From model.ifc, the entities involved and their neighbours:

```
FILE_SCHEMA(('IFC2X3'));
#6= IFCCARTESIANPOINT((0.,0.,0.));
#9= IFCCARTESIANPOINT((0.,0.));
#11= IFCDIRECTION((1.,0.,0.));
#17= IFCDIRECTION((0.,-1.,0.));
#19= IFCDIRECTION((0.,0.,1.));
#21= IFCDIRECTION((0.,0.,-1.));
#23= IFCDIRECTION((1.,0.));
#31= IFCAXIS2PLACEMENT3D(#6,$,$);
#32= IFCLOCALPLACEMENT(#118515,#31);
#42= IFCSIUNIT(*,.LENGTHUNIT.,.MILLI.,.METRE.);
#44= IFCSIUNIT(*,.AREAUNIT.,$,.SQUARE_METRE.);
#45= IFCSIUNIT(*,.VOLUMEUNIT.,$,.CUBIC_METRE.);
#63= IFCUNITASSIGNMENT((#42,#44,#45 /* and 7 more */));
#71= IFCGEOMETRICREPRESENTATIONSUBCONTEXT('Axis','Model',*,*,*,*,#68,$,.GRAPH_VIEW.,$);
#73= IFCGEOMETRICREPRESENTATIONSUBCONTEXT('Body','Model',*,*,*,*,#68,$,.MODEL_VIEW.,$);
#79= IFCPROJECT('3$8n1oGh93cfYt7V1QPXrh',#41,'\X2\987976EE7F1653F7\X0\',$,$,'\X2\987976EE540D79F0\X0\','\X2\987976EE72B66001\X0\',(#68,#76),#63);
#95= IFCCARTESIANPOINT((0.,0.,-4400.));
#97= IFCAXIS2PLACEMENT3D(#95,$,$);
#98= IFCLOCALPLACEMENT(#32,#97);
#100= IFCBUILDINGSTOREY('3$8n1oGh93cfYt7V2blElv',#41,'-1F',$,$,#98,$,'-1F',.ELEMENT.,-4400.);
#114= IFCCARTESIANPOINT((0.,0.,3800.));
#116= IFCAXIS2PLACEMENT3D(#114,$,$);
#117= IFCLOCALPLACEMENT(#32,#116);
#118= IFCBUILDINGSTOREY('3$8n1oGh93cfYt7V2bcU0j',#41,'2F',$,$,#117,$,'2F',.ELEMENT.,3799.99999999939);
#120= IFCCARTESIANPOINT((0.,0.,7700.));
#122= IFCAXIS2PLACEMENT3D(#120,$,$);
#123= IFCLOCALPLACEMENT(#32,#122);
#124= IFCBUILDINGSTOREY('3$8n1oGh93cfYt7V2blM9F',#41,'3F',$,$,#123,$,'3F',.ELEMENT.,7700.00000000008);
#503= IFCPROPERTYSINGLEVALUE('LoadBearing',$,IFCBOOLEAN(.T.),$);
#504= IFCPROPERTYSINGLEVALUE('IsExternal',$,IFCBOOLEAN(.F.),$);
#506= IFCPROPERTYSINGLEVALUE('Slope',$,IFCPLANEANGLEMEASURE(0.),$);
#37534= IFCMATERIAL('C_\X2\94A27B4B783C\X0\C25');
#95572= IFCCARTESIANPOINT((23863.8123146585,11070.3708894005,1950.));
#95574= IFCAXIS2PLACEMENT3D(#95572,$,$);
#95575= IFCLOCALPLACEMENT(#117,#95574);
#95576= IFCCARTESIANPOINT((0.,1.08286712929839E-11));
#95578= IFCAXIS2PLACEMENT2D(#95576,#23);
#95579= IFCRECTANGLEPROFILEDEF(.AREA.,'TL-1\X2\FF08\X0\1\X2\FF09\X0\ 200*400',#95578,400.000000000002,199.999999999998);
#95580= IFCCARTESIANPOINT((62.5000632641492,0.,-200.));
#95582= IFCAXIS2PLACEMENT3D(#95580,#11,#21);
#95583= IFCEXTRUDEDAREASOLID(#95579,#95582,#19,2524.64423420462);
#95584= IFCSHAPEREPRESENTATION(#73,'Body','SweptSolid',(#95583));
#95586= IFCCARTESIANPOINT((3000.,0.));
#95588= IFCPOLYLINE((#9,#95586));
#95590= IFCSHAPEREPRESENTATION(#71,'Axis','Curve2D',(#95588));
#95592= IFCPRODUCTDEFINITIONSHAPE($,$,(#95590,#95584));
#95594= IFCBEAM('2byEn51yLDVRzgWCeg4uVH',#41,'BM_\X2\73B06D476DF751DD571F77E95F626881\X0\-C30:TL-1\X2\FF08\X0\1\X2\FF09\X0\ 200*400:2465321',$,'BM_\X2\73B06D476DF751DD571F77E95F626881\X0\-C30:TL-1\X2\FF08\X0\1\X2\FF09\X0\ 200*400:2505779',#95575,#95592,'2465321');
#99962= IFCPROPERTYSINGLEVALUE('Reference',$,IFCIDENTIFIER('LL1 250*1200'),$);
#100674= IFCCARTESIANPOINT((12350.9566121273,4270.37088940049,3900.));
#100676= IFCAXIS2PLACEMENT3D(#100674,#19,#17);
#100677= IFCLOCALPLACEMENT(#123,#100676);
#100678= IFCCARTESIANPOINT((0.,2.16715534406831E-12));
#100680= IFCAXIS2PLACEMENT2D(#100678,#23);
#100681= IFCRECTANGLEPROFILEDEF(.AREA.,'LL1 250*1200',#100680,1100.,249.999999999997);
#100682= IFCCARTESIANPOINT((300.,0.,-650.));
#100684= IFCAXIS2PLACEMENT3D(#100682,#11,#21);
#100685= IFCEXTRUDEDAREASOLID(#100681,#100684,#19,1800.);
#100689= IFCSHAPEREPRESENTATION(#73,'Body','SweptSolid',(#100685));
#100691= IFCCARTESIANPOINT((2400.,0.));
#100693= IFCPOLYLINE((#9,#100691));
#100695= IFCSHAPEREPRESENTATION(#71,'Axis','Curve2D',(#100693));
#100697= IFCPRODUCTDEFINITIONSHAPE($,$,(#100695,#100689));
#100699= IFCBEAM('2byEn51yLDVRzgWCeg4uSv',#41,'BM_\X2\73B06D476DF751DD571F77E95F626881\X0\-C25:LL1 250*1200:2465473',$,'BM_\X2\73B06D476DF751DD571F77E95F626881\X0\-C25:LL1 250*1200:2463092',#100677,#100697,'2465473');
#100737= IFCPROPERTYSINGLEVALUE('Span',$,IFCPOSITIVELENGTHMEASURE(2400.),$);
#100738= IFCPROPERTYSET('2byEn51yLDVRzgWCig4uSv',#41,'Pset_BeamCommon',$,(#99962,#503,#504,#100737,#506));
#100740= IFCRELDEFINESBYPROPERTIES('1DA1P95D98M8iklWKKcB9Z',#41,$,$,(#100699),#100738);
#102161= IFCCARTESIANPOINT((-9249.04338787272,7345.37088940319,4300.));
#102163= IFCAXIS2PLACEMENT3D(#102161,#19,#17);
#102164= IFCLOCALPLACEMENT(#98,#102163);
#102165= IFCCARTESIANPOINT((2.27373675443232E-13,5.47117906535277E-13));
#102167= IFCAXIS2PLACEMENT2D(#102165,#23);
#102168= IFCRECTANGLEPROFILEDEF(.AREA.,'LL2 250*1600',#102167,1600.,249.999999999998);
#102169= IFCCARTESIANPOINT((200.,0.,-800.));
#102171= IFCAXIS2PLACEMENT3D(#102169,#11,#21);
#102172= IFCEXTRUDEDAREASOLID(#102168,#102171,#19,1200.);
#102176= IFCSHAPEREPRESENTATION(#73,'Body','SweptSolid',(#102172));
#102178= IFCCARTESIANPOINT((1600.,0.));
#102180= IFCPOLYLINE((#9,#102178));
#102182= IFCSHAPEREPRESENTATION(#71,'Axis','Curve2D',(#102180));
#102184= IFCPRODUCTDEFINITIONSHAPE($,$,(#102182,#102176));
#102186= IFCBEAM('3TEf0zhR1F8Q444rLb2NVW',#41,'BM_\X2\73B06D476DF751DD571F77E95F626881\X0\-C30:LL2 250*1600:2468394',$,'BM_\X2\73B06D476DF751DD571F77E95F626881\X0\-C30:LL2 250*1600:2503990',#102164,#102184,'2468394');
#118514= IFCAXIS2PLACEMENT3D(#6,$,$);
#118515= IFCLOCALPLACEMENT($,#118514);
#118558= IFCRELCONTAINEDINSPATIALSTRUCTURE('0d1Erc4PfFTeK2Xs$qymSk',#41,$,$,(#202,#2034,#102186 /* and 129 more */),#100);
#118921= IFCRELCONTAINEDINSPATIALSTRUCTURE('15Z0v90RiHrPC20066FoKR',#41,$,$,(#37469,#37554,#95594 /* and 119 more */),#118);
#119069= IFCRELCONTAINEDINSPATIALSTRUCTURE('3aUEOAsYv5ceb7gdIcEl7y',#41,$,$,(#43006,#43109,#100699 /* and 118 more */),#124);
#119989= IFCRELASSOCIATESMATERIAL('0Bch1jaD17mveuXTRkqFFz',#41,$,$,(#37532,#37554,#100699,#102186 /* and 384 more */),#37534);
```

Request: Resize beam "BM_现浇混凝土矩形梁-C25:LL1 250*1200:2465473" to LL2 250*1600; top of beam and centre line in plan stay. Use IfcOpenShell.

```python
import ifcopenshell
import ifcopenshell.api.pset
import ifcopenshell.util.element
import ifcopenshell.util.representation

model = ifcopenshell.open("model.ifc")

member = model.by_id(100699)
source = next(p for p in model.by_type("IfcRectangleProfileDef") if p.ProfileName == "LL2 250*1600")

body = ifcopenshell.util.representation.get_representation(member, "Model", "Body")
solid = body.Items[0]
old_profile = solid.SweptArea

# Copy the section's sizes but keep this member's own profile position.
profile = ifcopenshell.util.element.copy(model, source)
# Profiles are centred, so shift by half the change in depth to hold the top.
shift = (old_profile.XDim - profile.XDim) / 2
x, y = old_profile.Position.Location.Coordinates
up = (-1.0, 0.0)  # upwards, in the solid's own plane
location = model.createIfcCartesianPoint((x + up[0] * shift, y + up[1] * shift))
profile.Position = model.createIfcAxis2Placement2D(location, old_profile.Position.RefDirection)
solid.SweptArea = profile
if not model.get_total_inverses(old_profile):
    ifcopenshell.util.element.remove_deep2(model, old_profile)
member.Name = member.Name.replace("LL1 250*1200", "LL2 250*1600")
member.ObjectType = member.ObjectType.replace("LL1 250*1200", "LL2 250*1600")
pset = model.by_id(ifcopenshell.util.element.get_pset(member, "Pset_BeamCommon", should_inherit=False)["id"])
ifcopenshell.api.pset.edit_pset(model, pset=pset, properties={"Reference": "LL2 250*1600"})

print(solid.SweptArea)

model.write("model_updated.ifc")
```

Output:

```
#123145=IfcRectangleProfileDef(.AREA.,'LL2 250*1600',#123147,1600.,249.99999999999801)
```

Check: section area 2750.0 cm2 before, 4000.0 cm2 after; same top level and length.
